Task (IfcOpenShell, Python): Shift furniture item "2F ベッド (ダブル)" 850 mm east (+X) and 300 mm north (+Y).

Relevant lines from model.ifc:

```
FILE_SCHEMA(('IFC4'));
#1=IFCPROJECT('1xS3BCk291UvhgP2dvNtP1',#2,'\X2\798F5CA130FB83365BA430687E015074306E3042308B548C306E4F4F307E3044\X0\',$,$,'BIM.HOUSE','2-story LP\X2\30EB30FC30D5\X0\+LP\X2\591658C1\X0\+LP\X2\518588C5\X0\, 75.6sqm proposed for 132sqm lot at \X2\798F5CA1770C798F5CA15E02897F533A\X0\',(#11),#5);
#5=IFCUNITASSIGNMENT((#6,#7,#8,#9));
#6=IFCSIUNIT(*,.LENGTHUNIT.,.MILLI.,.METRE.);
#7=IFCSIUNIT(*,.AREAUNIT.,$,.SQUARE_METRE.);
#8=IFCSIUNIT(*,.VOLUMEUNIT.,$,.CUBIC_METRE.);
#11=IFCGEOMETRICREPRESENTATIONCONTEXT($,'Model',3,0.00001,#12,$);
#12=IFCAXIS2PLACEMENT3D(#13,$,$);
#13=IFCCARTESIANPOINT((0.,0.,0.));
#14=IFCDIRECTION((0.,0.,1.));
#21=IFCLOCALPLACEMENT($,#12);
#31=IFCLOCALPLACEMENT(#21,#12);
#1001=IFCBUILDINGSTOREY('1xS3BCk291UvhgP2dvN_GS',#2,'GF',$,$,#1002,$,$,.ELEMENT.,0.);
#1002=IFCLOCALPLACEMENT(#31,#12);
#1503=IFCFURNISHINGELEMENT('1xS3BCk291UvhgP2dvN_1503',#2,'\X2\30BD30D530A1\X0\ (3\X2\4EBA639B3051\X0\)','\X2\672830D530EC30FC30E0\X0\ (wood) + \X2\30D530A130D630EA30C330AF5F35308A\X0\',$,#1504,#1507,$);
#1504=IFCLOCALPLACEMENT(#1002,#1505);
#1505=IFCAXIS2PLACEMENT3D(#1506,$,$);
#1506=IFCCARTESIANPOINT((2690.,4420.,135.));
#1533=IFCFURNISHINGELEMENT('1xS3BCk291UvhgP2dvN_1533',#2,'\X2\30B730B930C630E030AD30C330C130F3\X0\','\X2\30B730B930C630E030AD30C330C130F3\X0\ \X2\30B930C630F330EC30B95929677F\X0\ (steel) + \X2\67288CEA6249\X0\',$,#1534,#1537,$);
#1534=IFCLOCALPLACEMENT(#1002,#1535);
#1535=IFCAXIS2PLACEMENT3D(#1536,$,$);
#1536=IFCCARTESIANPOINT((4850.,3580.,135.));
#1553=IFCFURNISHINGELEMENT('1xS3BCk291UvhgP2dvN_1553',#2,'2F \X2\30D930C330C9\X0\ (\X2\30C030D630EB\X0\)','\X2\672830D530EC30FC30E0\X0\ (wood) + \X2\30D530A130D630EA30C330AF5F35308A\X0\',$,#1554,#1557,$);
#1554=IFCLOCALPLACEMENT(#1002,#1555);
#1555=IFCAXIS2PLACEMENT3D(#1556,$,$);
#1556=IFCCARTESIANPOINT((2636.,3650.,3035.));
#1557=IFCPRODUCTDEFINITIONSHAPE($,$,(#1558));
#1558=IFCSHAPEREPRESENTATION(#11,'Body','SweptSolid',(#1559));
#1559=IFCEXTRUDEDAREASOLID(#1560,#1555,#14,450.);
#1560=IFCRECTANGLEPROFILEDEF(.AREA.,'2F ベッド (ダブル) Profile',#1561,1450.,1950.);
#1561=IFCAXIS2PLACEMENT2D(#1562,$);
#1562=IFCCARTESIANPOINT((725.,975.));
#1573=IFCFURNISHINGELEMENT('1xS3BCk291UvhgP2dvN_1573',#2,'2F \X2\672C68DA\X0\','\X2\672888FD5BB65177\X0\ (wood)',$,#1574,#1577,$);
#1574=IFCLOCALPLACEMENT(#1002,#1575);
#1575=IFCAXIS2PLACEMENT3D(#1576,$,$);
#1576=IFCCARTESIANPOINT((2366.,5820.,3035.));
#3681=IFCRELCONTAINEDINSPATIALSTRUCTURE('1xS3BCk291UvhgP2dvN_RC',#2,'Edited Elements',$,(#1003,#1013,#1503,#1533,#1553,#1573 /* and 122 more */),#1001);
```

```python
import ifcopenshell
import ifcopenshell.api.geometry
import ifcopenshell.util.placement
import ifcopenshell.util.unit

model = ifcopenshell.open("model.ifc")
unit_scale = ifcopenshell.util.unit.calculate_unit_scale(model)

item = model.by_id(1553)
matrix = ifcopenshell.util.placement.get_local_placement(item.ObjectPlacement)
matrix[0, 3] += 0.85 / unit_scale
matrix[1, 3] += 0.3 / unit_scale
ifcopenshell.api.geometry.edit_object_placement(model, product=item, matrix=matrix, is_si=False)

print(ifcopenshell.util.placement.get_local_placement(item.ObjectPlacement).round(3) + 0.0)

model.write("model-out.ifc")
```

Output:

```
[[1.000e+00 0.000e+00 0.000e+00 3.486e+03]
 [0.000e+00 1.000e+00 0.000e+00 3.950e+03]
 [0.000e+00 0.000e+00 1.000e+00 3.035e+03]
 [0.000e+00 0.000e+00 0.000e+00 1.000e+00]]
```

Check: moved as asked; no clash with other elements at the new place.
